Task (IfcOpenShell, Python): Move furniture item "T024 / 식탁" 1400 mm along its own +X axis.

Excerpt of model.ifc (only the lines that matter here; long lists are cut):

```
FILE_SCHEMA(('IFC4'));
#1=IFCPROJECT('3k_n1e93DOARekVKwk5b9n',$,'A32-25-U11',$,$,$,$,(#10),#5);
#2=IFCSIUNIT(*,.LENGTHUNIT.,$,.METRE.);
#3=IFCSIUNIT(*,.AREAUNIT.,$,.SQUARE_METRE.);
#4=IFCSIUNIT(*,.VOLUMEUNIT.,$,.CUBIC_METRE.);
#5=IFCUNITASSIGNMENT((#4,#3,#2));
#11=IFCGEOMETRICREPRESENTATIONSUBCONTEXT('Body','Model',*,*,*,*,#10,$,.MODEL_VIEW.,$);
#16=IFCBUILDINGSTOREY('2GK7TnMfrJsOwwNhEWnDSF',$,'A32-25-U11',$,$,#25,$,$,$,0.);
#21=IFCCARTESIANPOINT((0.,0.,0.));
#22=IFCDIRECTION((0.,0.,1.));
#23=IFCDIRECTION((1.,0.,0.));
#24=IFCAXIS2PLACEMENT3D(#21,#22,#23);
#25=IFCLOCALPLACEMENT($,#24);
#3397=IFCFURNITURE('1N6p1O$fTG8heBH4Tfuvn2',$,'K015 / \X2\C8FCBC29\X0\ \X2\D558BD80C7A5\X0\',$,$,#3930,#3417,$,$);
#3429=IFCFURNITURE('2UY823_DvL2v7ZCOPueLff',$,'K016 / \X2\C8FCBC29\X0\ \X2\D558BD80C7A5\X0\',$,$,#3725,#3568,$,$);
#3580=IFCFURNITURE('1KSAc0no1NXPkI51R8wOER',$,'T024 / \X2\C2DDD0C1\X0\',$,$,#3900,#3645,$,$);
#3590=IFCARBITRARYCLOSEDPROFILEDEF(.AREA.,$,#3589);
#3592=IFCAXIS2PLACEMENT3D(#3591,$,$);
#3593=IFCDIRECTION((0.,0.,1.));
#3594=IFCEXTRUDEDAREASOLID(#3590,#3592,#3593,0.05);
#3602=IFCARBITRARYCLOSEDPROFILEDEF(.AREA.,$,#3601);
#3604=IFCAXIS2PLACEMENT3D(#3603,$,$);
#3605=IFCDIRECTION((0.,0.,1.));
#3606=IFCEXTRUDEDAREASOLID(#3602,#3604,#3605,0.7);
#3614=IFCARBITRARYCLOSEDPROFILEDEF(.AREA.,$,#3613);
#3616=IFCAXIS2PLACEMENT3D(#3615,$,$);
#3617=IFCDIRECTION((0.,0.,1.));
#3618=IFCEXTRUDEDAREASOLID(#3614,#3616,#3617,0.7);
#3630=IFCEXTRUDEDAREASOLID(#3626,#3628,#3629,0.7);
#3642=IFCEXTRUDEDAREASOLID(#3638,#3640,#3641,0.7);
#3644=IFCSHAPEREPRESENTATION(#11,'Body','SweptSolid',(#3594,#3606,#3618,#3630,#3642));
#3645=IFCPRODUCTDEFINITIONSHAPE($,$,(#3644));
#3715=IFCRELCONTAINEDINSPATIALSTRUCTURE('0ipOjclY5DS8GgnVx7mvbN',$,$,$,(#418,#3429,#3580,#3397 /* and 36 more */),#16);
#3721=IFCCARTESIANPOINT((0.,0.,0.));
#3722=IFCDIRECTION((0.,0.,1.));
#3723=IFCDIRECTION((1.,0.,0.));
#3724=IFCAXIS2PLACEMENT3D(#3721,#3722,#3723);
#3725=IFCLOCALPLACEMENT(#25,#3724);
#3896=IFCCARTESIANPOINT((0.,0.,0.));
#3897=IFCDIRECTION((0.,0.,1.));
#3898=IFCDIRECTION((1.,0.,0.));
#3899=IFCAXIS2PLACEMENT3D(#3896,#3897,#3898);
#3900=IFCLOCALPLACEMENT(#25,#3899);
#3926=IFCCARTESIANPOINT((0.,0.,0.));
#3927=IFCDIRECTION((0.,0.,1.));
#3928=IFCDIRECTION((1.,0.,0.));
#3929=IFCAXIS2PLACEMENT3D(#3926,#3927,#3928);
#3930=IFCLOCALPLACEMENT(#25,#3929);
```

```python
import ifcopenshell
import ifcopenshell.api.geometry
import ifcopenshell.util.placement
import ifcopenshell.util.unit

model = ifcopenshell.open("model.ifc")
unit_scale = ifcopenshell.util.unit.calculate_unit_scale(model)

item = model.by_guid("1KSAc0no1NXPkI51R8wOER")
matrix = ifcopenshell.util.placement.get_local_placement(item.ObjectPlacement)
matrix[:3, 3] += matrix[:3, 0] * 1.4 / unit_scale
ifcopenshell.api.geometry.edit_object_placement(model, product=item, matrix=matrix, is_si=False)

print(ifcopenshell.util.placement.get_local_placement(item.ObjectPlacement).round(3) + 0.0)

model.write("model_v2.ifc")
```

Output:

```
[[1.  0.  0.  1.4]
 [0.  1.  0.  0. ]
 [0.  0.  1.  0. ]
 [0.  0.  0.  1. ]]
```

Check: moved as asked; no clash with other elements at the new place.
